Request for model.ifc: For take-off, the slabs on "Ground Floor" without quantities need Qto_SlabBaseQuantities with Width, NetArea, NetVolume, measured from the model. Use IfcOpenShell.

First a look at what the model holds.

```python
import ifcopenshell
import ifcopenshell.util.element
import ifcopenshell.util.unit

model = ifcopenshell.open("model.ifc")
print(model.schema)
for unit_type in ("LENGTHUNIT", "AREAUNIT", "VOLUMEUNIT"):
    print(unit_type, ifcopenshell.util.unit.calculate_unit_scale(model, unit_type))
storey = next(s for s in model.by_type("IfcBuildingStorey") if s.Name == "Ground Floor")
slabs = [e for e in ifcopenshell.util.element.get_decomposition(storey) if e.is_a("IfcSlab")]
for e in sorted(slabs, key=lambda e: e.id()):
    print(e.id(), e.is_a(), e.Name, list(ifcopenshell.util.element.get_psets(e, qtos_only=True)), sep=" | ")
```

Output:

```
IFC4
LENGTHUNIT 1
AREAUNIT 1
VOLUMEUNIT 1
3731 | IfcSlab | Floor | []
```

```python
import ifcopenshell
import ifcopenshell.api.pset
import ifcopenshell.geom
import ifcopenshell.util.element
import ifcopenshell.util.shape
import ifcopenshell.util.unit

model = ifcopenshell.open("model.ifc")
unit_scale = ifcopenshell.util.unit.calculate_unit_scale(model)
area_scale = ifcopenshell.util.unit.calculate_unit_scale(model, "AREAUNIT")
volume_scale = ifcopenshell.util.unit.calculate_unit_scale(model, "VOLUMEUNIT")
settings = ifcopenshell.geom.settings()

storey = next(s for s in model.by_type("IfcBuildingStorey") if s.Name == "Ground Floor")
slabs = [e for e in ifcopenshell.util.element.get_decomposition(storey) if e.is_a("IfcSlab")]

for e in sorted(slabs, key=lambda e: e.id()):
    if ifcopenshell.util.element.get_psets(e, qtos_only=True, should_inherit=False):
        continue
    # Geometry comes back in metres, in the element's own axes.
    shape = ifcopenshell.geom.create_shape(settings, e)
    values = {
        "Width": ifcopenshell.util.shape.get_z(shape.geometry) / unit_scale,
        "NetArea": ifcopenshell.util.shape.get_footprint_area(shape.geometry) / area_scale,
        "NetVolume": ifcopenshell.util.shape.get_volume(shape.geometry) / volume_scale,
    }
    qto = ifcopenshell.api.pset.add_qto(model, product=e, name="Qto_SlabBaseQuantities")
    ifcopenshell.api.pset.edit_qto(model, qto=qto, properties=values)
    print(e.id(), {k: round(v, 3) for k, v in values.items()})

model.write("model_rev.ifc")
```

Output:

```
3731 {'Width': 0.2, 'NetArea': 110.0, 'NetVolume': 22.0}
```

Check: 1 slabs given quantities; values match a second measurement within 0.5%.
